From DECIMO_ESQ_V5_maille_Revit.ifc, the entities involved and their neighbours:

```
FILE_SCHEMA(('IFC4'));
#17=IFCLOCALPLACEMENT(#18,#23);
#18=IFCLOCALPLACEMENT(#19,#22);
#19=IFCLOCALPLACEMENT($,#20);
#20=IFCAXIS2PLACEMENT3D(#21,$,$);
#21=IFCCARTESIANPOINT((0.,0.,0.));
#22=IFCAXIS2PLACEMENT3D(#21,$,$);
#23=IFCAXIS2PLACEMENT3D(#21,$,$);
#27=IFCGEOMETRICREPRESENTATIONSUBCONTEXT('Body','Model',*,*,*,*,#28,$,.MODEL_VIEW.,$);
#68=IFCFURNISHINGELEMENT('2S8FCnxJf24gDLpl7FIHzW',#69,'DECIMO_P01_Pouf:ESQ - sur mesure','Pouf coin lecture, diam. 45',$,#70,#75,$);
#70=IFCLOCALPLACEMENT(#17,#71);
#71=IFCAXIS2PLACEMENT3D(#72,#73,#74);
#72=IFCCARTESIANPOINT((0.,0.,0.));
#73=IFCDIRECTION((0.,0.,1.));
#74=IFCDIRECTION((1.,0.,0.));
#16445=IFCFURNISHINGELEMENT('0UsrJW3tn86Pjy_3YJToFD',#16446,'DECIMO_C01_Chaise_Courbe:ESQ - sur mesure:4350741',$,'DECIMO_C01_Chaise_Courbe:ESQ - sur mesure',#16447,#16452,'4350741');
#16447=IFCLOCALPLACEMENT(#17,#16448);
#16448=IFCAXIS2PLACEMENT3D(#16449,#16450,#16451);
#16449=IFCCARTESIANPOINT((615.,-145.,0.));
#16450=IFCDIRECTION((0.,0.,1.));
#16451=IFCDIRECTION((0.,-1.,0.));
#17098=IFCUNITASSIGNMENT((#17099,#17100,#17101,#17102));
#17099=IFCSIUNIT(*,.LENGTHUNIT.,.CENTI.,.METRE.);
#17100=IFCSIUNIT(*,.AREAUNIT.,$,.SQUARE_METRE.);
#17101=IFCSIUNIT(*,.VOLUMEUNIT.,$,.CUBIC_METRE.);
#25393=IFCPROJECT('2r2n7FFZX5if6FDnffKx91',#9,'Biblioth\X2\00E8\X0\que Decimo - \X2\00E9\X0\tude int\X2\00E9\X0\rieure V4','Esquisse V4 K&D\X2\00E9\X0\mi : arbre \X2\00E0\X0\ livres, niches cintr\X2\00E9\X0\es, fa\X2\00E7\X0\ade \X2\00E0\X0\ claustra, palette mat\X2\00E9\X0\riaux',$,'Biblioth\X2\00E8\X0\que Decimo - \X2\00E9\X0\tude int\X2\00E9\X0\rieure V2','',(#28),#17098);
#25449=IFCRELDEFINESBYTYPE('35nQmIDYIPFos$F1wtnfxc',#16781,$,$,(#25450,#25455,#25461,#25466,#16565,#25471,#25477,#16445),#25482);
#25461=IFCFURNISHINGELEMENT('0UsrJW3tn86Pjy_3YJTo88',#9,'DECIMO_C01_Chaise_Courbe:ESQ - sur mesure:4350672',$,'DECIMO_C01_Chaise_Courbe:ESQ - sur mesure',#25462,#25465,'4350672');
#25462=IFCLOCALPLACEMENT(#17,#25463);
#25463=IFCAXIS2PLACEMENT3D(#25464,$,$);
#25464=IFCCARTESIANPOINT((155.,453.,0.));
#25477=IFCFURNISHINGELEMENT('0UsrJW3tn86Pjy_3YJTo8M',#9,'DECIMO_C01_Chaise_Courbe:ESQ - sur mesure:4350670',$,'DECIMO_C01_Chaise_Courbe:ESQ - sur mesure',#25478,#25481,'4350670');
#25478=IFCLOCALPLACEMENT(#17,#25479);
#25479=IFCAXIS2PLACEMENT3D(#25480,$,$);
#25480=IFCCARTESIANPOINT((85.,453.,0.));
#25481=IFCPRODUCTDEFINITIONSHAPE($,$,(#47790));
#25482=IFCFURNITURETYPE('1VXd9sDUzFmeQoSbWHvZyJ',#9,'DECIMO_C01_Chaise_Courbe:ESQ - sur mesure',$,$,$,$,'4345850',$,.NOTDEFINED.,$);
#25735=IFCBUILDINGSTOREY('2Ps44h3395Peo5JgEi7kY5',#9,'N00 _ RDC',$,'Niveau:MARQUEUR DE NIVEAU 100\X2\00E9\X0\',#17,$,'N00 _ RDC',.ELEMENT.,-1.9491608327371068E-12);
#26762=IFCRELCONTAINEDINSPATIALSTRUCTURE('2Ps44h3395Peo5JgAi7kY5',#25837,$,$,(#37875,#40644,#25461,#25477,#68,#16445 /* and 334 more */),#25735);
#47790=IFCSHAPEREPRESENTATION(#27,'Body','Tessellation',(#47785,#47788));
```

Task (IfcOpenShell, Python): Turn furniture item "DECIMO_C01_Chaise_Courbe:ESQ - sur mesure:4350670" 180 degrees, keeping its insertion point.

```python
import ifcopenshell
import ifcopenshell.api.geometry
import ifcopenshell.util.placement

model = ifcopenshell.open("DECIMO_ESQ_V5_maille_Revit.ifc")

item = model.by_guid("0UsrJW3tn86Pjy_3YJTo8M")
matrix = ifcopenshell.util.placement.get_local_placement(item.ObjectPlacement)
matrix = matrix @ ifcopenshell.util.placement.rotation(180, "Z")
ifcopenshell.api.geometry.edit_object_placement(model, product=item, matrix=matrix, is_si=False)

print(ifcopenshell.util.placement.get_local_placement(item.ObjectPlacement).round(3) + 0.0)

model.write("DECIMO_ESQ_V5_maille_Revit_v2.ifc")
```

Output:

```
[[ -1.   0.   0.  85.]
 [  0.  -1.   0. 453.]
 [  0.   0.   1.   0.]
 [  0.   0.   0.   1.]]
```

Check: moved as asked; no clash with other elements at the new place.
